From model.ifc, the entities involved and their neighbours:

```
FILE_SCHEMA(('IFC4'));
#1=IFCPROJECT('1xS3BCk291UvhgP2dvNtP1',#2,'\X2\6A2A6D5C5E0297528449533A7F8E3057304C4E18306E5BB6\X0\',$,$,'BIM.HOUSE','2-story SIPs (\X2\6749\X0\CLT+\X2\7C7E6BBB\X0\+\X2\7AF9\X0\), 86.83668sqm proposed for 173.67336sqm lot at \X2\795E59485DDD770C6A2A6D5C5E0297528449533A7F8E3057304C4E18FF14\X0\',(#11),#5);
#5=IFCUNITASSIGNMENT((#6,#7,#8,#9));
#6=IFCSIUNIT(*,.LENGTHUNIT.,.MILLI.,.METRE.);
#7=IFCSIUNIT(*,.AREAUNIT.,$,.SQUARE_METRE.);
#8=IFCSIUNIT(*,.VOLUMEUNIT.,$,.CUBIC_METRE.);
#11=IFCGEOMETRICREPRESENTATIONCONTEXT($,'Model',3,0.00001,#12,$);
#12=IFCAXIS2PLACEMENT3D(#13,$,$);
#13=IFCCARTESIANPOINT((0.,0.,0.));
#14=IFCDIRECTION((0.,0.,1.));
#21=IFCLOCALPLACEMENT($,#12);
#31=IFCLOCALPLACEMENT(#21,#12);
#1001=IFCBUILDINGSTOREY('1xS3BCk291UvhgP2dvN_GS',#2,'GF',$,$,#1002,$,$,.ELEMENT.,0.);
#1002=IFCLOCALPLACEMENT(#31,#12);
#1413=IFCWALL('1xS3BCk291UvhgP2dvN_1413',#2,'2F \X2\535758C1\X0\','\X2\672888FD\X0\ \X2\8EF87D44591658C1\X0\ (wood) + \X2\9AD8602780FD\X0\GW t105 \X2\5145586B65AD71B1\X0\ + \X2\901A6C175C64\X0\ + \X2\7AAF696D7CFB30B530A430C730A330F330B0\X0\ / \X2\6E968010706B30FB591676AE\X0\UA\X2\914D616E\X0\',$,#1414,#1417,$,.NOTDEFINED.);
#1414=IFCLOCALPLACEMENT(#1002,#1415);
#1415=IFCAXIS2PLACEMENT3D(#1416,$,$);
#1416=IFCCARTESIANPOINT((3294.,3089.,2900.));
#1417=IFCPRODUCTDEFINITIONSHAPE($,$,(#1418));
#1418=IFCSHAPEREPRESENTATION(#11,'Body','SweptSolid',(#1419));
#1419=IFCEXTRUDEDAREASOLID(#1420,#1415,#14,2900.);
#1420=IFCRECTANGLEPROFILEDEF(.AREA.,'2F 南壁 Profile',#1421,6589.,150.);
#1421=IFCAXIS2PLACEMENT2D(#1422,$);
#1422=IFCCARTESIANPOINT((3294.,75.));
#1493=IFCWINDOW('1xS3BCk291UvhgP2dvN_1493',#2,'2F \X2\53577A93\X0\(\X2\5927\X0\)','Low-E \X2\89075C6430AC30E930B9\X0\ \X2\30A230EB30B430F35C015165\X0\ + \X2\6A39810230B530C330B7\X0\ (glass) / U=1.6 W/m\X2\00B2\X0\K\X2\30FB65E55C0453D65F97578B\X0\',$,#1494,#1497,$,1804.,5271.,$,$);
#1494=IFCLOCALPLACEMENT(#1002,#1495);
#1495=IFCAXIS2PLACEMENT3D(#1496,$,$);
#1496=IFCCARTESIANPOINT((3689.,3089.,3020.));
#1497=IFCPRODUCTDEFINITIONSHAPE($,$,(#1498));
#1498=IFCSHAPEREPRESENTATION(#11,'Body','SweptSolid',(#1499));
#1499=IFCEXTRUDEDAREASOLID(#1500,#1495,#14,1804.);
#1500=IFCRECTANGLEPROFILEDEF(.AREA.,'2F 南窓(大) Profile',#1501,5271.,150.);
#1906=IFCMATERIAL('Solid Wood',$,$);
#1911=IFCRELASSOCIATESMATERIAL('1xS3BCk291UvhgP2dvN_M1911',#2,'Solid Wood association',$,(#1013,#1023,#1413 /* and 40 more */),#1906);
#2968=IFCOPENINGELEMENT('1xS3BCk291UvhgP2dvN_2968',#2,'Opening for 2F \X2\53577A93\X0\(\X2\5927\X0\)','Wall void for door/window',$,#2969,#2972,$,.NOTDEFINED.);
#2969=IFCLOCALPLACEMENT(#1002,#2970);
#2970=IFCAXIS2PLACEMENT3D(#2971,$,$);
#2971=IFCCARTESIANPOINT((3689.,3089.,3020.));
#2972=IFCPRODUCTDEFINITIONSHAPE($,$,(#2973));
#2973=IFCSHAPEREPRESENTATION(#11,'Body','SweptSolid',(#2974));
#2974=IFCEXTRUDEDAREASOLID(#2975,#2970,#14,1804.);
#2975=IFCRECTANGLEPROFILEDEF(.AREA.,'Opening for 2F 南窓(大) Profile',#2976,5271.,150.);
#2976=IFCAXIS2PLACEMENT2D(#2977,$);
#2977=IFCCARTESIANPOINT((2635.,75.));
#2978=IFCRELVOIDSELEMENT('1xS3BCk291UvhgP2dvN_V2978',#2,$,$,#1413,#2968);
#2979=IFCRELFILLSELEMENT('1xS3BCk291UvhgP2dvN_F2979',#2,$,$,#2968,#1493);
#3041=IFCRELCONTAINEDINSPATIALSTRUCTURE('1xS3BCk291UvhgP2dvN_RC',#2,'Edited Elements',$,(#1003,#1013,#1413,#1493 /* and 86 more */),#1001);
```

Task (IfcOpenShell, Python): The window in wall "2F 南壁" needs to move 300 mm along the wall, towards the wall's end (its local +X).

```python
import ifcopenshell
import ifcopenshell.api.geometry
import ifcopenshell.util.placement
import ifcopenshell.util.unit

model = ifcopenshell.open("model.ifc")
unit_scale = ifcopenshell.util.unit.calculate_unit_scale(model)

window = model.by_guid("1xS3BCk291UvhgP2dvN_1493")
opening = window.FillsVoids[0].RelatingOpeningElement
wall = opening.VoidsElements[0].RelatingBuildingElement

wall_matrix = ifcopenshell.util.placement.get_local_placement(wall.ObjectPlacement)
shift = wall_matrix[:3, 0] * 0.3 / unit_scale
before = ifcopenshell.util.placement.get_local_placement(window.ObjectPlacement)[:3, 3].copy()

# The window is not placed relative to its opening, so move both.
for product in (opening, window):
    matrix = ifcopenshell.util.placement.get_local_placement(product.ObjectPlacement)
    matrix[:3, 3] += shift
    ifcopenshell.api.geometry.edit_object_placement(model, product=product, matrix=matrix, is_si=False)

after = ifcopenshell.util.placement.get_local_placement(window.ObjectPlacement)[:3, 3]
print("window moved by", (after - before).round(3) + 0.0)

model.write("model_edited.ifc")
```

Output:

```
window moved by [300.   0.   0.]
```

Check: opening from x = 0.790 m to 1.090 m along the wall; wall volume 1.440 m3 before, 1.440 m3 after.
